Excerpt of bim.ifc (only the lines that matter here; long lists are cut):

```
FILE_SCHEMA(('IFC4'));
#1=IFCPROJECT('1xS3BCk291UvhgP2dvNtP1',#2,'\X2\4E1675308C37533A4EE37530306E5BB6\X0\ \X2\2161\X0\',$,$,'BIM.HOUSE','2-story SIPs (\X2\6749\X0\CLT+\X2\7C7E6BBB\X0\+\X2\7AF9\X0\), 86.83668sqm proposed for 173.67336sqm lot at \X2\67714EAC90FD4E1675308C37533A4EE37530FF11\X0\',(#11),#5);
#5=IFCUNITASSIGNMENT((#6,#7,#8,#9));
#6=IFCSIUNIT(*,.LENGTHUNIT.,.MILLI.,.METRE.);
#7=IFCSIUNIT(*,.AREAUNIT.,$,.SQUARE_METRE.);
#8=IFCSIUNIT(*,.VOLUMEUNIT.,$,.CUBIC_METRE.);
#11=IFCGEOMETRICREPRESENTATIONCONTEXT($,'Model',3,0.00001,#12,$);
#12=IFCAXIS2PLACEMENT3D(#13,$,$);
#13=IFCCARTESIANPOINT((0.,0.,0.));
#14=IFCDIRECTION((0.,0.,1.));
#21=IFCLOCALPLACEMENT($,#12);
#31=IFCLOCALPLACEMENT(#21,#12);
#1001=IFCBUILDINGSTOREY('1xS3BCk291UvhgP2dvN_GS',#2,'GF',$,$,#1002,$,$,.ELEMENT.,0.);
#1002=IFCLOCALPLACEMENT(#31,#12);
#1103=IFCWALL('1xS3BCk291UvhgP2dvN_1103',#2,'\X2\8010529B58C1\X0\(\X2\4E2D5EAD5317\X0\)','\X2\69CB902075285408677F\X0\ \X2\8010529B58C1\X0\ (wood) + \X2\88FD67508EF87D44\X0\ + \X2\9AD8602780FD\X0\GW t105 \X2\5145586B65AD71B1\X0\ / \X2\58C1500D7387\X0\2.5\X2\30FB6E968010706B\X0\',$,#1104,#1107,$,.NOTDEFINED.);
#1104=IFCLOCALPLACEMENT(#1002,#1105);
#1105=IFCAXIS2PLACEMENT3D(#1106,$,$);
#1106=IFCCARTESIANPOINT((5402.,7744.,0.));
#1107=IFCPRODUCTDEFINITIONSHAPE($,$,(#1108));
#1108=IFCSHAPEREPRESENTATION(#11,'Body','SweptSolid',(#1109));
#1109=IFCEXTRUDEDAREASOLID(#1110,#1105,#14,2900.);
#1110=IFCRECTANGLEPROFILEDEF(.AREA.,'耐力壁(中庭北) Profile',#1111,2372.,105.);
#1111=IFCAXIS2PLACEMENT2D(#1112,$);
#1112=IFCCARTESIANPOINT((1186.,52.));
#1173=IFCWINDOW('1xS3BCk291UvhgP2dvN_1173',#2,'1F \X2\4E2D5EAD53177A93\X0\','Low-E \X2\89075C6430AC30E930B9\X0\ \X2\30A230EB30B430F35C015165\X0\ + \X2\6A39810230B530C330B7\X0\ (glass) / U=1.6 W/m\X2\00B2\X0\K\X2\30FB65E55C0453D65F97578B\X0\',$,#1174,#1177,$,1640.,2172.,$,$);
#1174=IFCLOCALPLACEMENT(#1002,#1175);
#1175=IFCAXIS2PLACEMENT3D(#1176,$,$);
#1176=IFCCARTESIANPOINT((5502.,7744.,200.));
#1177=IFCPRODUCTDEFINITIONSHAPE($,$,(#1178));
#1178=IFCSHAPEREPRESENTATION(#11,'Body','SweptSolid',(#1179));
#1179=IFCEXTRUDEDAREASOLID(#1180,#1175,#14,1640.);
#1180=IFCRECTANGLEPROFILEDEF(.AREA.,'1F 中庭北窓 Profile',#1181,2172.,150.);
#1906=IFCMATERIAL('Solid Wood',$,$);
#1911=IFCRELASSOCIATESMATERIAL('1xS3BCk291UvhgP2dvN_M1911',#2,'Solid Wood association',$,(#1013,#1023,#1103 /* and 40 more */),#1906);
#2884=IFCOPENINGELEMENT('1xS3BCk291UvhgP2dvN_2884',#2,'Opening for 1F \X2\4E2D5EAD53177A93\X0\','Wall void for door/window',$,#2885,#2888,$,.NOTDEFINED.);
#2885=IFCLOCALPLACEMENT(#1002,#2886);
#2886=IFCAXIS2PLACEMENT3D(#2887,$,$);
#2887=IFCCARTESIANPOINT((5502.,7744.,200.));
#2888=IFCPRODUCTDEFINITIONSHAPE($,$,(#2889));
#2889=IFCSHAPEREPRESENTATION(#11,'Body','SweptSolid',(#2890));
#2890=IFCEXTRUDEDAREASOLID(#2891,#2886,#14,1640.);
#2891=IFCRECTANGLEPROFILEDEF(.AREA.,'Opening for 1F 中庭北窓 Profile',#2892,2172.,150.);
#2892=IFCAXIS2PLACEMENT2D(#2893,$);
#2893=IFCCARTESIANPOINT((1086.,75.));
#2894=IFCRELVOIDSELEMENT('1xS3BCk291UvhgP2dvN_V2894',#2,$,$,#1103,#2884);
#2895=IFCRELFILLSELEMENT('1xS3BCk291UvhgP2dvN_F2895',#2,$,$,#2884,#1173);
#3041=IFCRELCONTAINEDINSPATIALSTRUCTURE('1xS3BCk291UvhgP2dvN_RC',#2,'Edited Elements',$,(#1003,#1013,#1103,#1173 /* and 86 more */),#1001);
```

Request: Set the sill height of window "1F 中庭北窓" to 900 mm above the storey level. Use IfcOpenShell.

```python
import numpy as np
import ifcopenshell
import ifcopenshell.api.geometry
import ifcopenshell.geom
import ifcopenshell.util.element
import ifcopenshell.util.placement
import ifcopenshell.util.shape
import ifcopenshell.util.unit

model = ifcopenshell.open("bim.ifc")
unit_scale = ifcopenshell.util.unit.calculate_unit_scale(model)

window = model.by_id(1173)
opening = window.FillsVoids[0].RelatingOpeningElement
storey = ifcopenshell.util.element.get_container(window, ifc_class="IfcBuildingStorey")
level = ifcopenshell.util.placement.get_local_placement(storey.ObjectPlacement)[2, 3]

# The opening's origin need not be at the sill, so measure its lowest point.
shape = ifcopenshell.geom.create_shape(ifcopenshell.geom.settings(), opening)
bottom = ifcopenshell.util.shape.get_shape_bottom_elevation(shape, shape.geometry) / unit_scale
dz = level + 0.9 / unit_scale - bottom

shift = np.array([0.0, 0.0, dz])
# The window is not placed relative to its opening, so move both.
for product in (opening, window):
    matrix = ifcopenshell.util.placement.get_local_placement(product.ObjectPlacement)
    matrix[:3, 3] += shift
    ifcopenshell.api.geometry.edit_object_placement(model, product=product, matrix=matrix, is_si=False)

print(f"moved by {dz * unit_scale:+.3f} m")

model.write("bim_updated.ifc")
```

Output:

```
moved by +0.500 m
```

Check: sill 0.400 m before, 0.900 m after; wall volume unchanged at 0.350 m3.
